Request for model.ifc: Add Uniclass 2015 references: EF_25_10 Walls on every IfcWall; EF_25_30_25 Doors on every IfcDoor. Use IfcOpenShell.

First a look at what the model holds.

```python
import ifcopenshell

model = ifcopenshell.open("model.ifc")
print(model.schema)
print("classifications:", [c.Name for c in model.by_type("IfcClassification")])
for ifc_class in ("IfcDoor", "IfcRoof", "IfcStair", "IfcWall", "IfcWindow"):
    print(ifc_class, len(model.by_type(ifc_class)))
```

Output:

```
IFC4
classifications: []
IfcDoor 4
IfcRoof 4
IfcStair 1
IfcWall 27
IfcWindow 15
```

```python
import ifcopenshell
import ifcopenshell.api.classification

model = ifcopenshell.open("model.ifc")

system = ifcopenshell.api.classification.add_classification(model, classification="Uniclass 2015")

codes = {
    "IfcWall": ("EF_25_10", "Walls"),
    "IfcDoor": ("EF_25_30_25", "Doors"),
}
for ifc_class, (code, name) in codes.items():
    products = model.by_type(ifc_class)
    ifcopenshell.api.classification.add_reference(
        model, products=products, classification=system, identification=code, name=name
    )
    print(code, len(products))

model.write("model_updated.ifc")
```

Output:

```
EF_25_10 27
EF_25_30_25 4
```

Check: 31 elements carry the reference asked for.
